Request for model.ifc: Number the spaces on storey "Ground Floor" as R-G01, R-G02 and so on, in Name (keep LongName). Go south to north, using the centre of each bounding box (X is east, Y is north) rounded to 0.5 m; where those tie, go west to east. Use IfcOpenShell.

First a look at what the model holds.

```python
import ifcopenshell
import ifcopenshell.util.element
import ifcopenshell.util.placement

model = ifcopenshell.open("model.ifc")
print(model.schema)
storey = next(s for s in model.by_type("IfcBuildingStorey") if s.Name == "Ground Floor")
spaces = [e for e in ifcopenshell.util.element.get_decomposition(storey) if e.is_a("IfcSpace")]
for e in sorted(spaces, key=lambda e: e.id()):
    origin = ifcopenshell.util.placement.get_local_placement(e.ObjectPlacement)[:3, 3]
    print(e.id(), e.Name, e.LongName, origin.round(2) + 0.0, sep=" | ")
```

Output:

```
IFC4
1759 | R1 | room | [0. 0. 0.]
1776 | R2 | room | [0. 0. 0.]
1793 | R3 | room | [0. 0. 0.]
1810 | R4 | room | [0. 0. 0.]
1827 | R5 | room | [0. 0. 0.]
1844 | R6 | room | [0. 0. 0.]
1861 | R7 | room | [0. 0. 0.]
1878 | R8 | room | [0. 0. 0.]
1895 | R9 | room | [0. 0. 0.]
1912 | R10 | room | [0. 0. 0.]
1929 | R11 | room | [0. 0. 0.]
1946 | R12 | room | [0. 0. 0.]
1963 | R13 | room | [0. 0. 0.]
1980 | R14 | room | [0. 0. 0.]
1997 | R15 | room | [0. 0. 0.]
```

```python
import ifcopenshell
import ifcopenshell.geom
import ifcopenshell.util.element
import ifcopenshell.util.shape

model = ifcopenshell.open("model.ifc")
settings = ifcopenshell.geom.settings()
settings.set("use-world-coords", True)


def centre(element):
    shape = ifcopenshell.geom.create_shape(settings, element)
    return ifcopenshell.util.shape.get_bbox_centroid(shape.geometry)


storey = next(s for s in model.by_type("IfcBuildingStorey") if s.Name == "Ground Floor")
spaces = [e for e in ifcopenshell.util.element.get_decomposition(storey) if e.is_a("IfcSpace")]

# Insertion points can sit at a corner or the storey origin, so sort by the geometry (in metres).
centres = {e: centre(e) for e in spaces}
spaces.sort(key=lambda e: (round(centres[e][1] / 0.5), centres[e][0]))

for i, e in enumerate(spaces, start=1):
    number = f"R-G{i:02d}"
    e.Name = number
    print(e.id(), number)

model.write("model-out.ifc")
```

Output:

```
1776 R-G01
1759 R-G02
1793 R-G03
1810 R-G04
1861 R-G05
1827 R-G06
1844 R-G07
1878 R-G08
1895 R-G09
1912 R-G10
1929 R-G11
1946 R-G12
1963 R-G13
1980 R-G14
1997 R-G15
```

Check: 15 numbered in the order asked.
